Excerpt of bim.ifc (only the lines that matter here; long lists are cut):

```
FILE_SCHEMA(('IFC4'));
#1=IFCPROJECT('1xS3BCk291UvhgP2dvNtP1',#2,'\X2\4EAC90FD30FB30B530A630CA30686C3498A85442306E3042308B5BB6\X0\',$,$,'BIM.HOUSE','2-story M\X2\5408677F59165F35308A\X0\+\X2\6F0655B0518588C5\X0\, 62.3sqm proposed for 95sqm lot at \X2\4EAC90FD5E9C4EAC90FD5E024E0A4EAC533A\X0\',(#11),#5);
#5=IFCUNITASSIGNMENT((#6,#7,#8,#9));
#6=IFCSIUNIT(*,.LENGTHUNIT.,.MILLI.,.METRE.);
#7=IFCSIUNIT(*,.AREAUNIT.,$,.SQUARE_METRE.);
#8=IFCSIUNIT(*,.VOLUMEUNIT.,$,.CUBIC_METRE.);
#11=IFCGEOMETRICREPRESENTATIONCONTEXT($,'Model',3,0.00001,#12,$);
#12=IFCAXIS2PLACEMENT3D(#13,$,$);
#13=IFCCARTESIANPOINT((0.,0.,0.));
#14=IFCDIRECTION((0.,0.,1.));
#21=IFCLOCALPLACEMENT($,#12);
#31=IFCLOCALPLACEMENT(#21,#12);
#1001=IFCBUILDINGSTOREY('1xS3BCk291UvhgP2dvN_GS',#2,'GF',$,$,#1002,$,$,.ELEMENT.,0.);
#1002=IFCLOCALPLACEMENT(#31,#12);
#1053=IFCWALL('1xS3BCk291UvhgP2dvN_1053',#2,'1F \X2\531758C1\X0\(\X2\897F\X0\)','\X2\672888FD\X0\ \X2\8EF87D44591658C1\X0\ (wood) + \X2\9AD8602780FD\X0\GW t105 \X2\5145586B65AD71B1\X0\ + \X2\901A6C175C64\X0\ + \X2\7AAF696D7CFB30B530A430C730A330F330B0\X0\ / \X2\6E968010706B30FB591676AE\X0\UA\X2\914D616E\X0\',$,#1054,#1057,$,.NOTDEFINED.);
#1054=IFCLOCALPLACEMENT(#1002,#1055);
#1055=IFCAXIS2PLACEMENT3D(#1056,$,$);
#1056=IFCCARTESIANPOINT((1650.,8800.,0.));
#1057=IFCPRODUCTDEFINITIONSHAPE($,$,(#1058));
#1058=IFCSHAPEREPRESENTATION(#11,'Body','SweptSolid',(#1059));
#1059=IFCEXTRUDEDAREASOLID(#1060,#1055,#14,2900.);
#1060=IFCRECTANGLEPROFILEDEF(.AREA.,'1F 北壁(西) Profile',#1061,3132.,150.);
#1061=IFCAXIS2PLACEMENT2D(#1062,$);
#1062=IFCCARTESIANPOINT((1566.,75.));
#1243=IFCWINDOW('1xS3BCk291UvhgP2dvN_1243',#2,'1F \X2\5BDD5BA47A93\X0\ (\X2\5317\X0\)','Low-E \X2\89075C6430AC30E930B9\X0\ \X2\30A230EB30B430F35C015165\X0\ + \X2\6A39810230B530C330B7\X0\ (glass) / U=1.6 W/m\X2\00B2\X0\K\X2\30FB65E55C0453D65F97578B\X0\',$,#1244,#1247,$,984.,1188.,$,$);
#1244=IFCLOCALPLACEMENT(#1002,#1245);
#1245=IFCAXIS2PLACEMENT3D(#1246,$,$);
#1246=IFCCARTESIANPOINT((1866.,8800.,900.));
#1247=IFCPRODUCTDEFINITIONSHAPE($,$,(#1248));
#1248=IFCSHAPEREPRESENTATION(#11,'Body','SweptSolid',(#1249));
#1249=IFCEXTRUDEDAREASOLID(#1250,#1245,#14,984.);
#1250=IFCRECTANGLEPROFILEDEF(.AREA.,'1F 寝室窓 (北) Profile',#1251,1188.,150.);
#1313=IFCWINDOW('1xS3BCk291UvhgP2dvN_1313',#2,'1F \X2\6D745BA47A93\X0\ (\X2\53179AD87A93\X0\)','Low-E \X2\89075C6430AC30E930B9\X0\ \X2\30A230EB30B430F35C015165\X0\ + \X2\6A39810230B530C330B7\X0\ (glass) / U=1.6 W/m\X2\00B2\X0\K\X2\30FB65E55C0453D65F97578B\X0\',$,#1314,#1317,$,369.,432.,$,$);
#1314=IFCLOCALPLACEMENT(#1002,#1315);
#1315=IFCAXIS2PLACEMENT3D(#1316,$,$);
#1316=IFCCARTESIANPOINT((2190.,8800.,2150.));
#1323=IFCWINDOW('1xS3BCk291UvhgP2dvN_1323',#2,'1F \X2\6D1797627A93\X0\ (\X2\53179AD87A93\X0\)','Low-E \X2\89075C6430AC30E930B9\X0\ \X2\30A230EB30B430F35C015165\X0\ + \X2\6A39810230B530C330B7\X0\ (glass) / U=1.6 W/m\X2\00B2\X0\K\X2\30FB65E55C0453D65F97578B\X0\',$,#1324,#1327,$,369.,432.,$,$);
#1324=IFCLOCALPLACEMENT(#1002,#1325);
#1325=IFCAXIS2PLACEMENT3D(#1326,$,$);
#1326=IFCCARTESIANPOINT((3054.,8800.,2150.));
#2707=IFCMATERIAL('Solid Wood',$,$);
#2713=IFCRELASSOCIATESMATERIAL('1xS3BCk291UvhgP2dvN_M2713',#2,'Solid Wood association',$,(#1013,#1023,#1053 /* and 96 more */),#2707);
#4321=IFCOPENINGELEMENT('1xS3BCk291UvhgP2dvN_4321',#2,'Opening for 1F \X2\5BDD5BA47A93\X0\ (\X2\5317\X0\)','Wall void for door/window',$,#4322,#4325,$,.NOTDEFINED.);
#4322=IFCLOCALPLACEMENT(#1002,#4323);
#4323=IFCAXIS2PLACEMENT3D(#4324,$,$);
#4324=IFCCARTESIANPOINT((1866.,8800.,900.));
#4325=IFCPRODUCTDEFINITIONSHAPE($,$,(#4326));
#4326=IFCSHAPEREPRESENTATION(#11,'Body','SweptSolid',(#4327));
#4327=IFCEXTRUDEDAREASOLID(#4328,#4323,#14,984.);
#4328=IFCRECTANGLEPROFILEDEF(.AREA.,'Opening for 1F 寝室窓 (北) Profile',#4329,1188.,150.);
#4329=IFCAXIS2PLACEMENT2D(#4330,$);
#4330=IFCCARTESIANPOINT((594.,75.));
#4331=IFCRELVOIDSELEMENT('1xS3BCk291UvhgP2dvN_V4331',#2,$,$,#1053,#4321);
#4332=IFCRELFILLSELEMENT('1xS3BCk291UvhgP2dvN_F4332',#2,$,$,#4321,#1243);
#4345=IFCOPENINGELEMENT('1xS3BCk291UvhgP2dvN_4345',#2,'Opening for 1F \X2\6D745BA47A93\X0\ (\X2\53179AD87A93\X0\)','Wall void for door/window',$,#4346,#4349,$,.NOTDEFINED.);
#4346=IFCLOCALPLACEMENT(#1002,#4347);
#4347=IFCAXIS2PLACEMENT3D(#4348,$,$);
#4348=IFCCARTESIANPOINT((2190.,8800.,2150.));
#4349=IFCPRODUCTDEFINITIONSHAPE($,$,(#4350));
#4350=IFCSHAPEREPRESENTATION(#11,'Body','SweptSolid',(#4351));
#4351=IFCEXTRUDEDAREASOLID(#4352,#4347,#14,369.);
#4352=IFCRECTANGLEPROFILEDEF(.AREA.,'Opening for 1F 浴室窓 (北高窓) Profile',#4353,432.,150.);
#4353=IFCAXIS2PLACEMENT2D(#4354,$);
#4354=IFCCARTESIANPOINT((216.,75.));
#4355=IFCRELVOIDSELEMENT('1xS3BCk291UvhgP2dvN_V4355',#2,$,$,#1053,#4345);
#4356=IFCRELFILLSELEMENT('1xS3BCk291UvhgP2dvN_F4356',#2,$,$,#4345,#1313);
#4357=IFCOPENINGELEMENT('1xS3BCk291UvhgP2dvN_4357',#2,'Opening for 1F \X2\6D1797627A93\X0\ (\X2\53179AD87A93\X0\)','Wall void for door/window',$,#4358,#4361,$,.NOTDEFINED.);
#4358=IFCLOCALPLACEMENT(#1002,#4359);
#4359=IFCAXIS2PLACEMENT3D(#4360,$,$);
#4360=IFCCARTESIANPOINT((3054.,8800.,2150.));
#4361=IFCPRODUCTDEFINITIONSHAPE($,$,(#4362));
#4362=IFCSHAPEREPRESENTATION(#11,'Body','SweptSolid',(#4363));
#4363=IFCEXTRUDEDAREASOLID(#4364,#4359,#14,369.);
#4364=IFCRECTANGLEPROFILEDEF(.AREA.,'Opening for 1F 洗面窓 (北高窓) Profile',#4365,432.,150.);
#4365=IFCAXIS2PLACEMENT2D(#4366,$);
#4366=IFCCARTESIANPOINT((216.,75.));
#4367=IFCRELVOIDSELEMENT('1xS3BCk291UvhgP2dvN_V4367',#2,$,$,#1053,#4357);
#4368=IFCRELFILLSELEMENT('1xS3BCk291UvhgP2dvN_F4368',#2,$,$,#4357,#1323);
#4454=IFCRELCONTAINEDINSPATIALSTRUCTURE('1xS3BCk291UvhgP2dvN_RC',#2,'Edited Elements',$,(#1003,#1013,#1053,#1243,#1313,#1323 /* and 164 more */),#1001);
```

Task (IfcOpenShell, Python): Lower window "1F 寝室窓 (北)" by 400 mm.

```python
import numpy as np
import ifcopenshell
import ifcopenshell.api.geometry
import ifcopenshell.util.placement
import ifcopenshell.util.unit

model = ifcopenshell.open("bim.ifc")
unit_scale = ifcopenshell.util.unit.calculate_unit_scale(model)

window = model.by_id(1243)
opening = window.FillsVoids[0].RelatingOpeningElement
dz = -0.4 / unit_scale

shift = np.array([0.0, 0.0, dz])
# The window is not placed relative to its opening, so move both.
for product in (opening, window):
    matrix = ifcopenshell.util.placement.get_local_placement(product.ObjectPlacement)
    matrix[:3, 3] += shift
    ifcopenshell.api.geometry.edit_object_placement(model, product=product, matrix=matrix, is_si=False)

print(f"moved by {dz * unit_scale:+.3f} m")

model.write("bim_updated.ifc")
```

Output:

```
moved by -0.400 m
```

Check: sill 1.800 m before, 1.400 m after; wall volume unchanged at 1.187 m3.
